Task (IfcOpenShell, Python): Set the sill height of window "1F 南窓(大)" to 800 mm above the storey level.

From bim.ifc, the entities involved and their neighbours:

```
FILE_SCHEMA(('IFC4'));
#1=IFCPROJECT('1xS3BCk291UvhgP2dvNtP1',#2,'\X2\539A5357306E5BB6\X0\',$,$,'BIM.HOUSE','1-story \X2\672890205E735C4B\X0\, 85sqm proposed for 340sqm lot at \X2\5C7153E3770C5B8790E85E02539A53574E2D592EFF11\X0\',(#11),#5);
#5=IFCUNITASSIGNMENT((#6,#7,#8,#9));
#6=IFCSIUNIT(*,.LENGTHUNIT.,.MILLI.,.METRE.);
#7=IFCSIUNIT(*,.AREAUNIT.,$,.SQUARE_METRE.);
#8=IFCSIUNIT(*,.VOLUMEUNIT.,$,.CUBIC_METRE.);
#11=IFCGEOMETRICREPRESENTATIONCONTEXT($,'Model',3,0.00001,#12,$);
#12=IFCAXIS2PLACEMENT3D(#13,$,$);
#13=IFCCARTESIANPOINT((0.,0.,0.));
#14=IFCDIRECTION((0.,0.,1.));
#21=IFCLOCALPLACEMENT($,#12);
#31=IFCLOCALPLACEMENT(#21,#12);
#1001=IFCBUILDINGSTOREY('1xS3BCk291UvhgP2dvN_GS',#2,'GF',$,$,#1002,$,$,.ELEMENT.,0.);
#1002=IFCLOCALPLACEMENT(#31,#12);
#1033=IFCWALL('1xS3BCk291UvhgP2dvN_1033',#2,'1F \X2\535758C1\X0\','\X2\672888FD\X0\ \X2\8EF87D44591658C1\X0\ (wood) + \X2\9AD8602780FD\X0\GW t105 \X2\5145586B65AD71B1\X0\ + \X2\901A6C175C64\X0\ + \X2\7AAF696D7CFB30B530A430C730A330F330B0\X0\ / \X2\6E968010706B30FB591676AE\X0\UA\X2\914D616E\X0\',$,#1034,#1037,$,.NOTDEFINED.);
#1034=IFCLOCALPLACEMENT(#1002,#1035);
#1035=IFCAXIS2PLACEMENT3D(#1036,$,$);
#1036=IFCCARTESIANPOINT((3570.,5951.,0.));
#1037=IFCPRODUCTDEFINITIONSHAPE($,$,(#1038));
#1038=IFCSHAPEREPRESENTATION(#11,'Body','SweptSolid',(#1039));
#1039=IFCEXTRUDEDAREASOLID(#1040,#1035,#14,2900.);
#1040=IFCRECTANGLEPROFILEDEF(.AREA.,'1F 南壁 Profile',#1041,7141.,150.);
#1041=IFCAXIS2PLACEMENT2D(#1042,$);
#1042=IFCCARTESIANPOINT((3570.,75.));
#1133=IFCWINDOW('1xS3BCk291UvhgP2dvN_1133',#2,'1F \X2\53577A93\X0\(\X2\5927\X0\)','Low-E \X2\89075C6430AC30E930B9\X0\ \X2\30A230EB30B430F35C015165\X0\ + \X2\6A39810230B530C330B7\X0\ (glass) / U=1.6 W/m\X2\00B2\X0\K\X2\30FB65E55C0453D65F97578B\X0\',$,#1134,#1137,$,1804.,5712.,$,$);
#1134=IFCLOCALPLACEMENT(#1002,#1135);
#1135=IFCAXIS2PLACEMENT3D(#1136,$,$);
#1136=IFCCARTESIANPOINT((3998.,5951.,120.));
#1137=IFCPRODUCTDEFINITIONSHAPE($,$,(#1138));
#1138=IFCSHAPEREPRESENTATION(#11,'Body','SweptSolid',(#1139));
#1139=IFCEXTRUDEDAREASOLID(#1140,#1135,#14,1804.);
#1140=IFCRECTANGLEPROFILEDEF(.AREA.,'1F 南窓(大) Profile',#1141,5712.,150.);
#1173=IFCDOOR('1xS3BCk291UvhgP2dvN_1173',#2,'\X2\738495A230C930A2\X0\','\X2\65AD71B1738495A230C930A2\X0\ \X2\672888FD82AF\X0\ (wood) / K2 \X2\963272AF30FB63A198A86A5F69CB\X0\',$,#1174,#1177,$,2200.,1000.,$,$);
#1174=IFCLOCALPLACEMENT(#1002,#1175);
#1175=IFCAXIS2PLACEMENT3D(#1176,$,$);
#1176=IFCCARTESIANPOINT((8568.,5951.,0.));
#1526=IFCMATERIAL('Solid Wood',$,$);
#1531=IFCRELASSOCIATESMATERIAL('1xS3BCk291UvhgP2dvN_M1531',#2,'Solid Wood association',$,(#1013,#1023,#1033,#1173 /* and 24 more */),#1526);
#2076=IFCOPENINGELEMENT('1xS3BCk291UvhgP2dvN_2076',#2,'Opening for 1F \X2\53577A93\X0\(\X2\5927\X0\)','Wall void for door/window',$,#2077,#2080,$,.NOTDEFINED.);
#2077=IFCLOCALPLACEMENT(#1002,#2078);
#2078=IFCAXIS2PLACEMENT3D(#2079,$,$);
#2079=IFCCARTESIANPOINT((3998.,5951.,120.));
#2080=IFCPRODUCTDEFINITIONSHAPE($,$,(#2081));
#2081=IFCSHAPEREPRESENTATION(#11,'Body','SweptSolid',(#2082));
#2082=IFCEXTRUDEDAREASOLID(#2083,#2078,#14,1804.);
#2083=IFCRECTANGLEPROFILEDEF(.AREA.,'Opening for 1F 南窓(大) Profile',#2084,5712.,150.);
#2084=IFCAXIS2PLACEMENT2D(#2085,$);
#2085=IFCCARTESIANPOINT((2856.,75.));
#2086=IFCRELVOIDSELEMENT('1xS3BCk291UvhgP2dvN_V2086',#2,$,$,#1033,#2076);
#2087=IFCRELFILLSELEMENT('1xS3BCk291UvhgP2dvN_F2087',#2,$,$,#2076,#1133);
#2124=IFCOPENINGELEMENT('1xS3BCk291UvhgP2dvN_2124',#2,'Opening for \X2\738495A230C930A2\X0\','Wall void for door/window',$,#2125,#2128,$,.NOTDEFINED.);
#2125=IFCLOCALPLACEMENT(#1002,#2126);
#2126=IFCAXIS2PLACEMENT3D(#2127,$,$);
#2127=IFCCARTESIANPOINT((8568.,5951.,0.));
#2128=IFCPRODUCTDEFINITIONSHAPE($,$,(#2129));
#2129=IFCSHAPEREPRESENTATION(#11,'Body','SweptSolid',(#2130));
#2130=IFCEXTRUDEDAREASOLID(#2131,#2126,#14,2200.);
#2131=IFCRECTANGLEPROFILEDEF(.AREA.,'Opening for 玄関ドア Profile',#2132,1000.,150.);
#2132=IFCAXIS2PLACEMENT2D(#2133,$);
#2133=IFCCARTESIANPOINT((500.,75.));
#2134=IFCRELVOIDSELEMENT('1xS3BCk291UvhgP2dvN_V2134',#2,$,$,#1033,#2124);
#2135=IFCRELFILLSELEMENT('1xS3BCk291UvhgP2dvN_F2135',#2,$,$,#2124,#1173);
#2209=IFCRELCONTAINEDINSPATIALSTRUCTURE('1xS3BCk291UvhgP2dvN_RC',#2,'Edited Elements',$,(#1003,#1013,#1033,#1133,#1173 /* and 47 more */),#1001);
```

```python
import numpy as np
import ifcopenshell
import ifcopenshell.api.geometry
import ifcopenshell.geom
import ifcopenshell.util.element
import ifcopenshell.util.placement
import ifcopenshell.util.shape
import ifcopenshell.util.unit

model = ifcopenshell.open("bim.ifc")
unit_scale = ifcopenshell.util.unit.calculate_unit_scale(model)

window = model.by_guid("1xS3BCk291UvhgP2dvN_1133")
opening = window.FillsVoids[0].RelatingOpeningElement
storey = ifcopenshell.util.element.get_container(window, ifc_class="IfcBuildingStorey")
level = ifcopenshell.util.placement.get_local_placement(storey.ObjectPlacement)[2, 3]

# The opening's origin need not be at the sill, so measure its lowest point.
shape = ifcopenshell.geom.create_shape(ifcopenshell.geom.settings(), opening)
bottom = ifcopenshell.util.shape.get_shape_bottom_elevation(shape, shape.geometry) / unit_scale
dz = level + 800.0 - bottom

shift = np.array([0.0, 0.0, dz])
# The window is not placed relative to its opening, so move both.
for product in (opening, window):
    matrix = ifcopenshell.util.placement.get_local_placement(product.ObjectPlacement)
    matrix[:3, 3] += shift
    ifcopenshell.api.geometry.edit_object_placement(model, product=product, matrix=matrix, is_si=False)

print(f"moved by {dz * unit_scale:+.3f} m")

model.write("bim_v2.ifc")
```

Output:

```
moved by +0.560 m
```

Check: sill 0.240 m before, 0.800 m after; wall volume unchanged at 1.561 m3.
